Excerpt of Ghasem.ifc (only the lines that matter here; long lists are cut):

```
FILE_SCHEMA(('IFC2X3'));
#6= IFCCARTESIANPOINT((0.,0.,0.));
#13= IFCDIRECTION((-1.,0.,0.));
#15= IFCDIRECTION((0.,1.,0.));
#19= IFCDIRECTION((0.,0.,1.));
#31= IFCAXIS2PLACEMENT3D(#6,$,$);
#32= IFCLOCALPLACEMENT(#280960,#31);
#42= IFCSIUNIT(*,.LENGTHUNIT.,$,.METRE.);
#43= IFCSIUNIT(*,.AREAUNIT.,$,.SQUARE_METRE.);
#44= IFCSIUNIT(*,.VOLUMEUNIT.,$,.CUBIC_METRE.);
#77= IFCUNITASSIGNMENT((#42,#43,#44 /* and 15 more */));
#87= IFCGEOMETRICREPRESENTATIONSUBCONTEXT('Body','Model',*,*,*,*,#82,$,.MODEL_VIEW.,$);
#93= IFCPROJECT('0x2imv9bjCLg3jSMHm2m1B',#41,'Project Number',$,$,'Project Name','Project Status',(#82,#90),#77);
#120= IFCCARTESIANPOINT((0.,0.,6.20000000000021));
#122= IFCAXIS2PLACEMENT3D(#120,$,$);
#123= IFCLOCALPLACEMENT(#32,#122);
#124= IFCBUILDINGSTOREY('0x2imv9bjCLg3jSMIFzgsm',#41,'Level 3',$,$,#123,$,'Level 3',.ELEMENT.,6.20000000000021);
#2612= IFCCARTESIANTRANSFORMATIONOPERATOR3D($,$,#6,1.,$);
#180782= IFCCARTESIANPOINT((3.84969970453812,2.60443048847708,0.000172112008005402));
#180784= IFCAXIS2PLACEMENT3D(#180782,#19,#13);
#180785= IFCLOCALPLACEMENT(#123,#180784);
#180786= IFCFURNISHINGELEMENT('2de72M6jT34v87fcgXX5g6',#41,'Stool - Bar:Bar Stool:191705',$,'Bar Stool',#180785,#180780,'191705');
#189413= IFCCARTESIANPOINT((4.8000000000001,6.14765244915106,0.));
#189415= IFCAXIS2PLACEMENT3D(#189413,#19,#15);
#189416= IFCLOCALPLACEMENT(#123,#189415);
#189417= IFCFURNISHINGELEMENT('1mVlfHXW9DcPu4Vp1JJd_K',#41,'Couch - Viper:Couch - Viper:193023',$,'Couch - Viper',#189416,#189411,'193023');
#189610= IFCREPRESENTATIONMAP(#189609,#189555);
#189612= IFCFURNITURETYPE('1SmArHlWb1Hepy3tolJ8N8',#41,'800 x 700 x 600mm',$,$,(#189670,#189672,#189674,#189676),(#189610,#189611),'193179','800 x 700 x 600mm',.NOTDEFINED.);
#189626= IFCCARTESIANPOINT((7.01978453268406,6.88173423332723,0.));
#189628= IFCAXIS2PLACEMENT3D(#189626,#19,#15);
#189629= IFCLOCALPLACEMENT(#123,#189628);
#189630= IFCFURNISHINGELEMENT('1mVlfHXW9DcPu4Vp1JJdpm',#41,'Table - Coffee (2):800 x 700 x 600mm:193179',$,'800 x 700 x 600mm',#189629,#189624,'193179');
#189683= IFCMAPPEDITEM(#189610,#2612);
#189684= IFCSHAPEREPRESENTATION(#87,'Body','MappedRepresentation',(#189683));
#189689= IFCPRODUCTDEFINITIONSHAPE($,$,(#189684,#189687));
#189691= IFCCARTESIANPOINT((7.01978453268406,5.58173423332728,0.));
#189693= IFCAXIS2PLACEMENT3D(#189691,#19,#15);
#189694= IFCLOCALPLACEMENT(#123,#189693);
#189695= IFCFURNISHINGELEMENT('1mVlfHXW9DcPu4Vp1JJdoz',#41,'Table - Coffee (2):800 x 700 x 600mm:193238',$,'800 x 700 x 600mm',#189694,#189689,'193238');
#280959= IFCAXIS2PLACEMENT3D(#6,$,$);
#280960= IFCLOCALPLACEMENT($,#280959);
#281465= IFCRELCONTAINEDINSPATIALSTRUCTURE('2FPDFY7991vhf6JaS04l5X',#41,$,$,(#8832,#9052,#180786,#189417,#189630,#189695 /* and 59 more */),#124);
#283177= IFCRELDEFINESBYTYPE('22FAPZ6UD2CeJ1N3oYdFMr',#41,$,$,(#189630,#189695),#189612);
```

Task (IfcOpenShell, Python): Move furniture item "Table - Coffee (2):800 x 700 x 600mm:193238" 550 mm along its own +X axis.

```python
import ifcopenshell
import ifcopenshell.api.geometry
import ifcopenshell.util.placement
import ifcopenshell.util.unit

model = ifcopenshell.open("Ghasem.ifc")
unit_scale = ifcopenshell.util.unit.calculate_unit_scale(model)

item = model.by_guid("1mVlfHXW9DcPu4Vp1JJdoz")
matrix = ifcopenshell.util.placement.get_local_placement(item.ObjectPlacement)
matrix[:3, 3] += matrix[:3, 0] * 0.55 / unit_scale
ifcopenshell.api.geometry.edit_object_placement(model, product=item, matrix=matrix, is_si=False)

print(ifcopenshell.util.placement.get_local_placement(item.ObjectPlacement).round(3) + 0.0)

model.write("Ghasem_v2.ifc")
```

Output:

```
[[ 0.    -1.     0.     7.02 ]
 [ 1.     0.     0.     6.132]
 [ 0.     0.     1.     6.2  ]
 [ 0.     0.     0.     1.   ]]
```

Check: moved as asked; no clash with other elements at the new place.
